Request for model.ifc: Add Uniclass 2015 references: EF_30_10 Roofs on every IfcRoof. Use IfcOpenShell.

First a look at what the model holds.

```python
import ifcopenshell

model = ifcopenshell.open("model.ifc")
print(model.schema)
print("classifications:", [c.Name for c in model.by_type("IfcClassification")])
for ifc_class in ("IfcDoor", "IfcRoof", "IfcStair", "IfcWall", "IfcWindow"):
    print(ifc_class, len(model.by_type(ifc_class)))
```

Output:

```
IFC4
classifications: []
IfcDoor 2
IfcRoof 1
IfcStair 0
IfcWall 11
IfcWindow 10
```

```python
import ifcopenshell
import ifcopenshell.api.classification

model = ifcopenshell.open("model.ifc")

system = ifcopenshell.api.classification.add_classification(model, classification="Uniclass 2015")

codes = {
    "IfcRoof": ("EF_30_10", "Roofs"),
}
for ifc_class, (code, name) in codes.items():
    products = model.by_type(ifc_class)
    ifcopenshell.api.classification.add_reference(
        model, products=products, classification=system, identification=code, name=name
    )
    print(code, len(products))

model.write("model_rev.ifc")
```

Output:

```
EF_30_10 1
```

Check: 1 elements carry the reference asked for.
